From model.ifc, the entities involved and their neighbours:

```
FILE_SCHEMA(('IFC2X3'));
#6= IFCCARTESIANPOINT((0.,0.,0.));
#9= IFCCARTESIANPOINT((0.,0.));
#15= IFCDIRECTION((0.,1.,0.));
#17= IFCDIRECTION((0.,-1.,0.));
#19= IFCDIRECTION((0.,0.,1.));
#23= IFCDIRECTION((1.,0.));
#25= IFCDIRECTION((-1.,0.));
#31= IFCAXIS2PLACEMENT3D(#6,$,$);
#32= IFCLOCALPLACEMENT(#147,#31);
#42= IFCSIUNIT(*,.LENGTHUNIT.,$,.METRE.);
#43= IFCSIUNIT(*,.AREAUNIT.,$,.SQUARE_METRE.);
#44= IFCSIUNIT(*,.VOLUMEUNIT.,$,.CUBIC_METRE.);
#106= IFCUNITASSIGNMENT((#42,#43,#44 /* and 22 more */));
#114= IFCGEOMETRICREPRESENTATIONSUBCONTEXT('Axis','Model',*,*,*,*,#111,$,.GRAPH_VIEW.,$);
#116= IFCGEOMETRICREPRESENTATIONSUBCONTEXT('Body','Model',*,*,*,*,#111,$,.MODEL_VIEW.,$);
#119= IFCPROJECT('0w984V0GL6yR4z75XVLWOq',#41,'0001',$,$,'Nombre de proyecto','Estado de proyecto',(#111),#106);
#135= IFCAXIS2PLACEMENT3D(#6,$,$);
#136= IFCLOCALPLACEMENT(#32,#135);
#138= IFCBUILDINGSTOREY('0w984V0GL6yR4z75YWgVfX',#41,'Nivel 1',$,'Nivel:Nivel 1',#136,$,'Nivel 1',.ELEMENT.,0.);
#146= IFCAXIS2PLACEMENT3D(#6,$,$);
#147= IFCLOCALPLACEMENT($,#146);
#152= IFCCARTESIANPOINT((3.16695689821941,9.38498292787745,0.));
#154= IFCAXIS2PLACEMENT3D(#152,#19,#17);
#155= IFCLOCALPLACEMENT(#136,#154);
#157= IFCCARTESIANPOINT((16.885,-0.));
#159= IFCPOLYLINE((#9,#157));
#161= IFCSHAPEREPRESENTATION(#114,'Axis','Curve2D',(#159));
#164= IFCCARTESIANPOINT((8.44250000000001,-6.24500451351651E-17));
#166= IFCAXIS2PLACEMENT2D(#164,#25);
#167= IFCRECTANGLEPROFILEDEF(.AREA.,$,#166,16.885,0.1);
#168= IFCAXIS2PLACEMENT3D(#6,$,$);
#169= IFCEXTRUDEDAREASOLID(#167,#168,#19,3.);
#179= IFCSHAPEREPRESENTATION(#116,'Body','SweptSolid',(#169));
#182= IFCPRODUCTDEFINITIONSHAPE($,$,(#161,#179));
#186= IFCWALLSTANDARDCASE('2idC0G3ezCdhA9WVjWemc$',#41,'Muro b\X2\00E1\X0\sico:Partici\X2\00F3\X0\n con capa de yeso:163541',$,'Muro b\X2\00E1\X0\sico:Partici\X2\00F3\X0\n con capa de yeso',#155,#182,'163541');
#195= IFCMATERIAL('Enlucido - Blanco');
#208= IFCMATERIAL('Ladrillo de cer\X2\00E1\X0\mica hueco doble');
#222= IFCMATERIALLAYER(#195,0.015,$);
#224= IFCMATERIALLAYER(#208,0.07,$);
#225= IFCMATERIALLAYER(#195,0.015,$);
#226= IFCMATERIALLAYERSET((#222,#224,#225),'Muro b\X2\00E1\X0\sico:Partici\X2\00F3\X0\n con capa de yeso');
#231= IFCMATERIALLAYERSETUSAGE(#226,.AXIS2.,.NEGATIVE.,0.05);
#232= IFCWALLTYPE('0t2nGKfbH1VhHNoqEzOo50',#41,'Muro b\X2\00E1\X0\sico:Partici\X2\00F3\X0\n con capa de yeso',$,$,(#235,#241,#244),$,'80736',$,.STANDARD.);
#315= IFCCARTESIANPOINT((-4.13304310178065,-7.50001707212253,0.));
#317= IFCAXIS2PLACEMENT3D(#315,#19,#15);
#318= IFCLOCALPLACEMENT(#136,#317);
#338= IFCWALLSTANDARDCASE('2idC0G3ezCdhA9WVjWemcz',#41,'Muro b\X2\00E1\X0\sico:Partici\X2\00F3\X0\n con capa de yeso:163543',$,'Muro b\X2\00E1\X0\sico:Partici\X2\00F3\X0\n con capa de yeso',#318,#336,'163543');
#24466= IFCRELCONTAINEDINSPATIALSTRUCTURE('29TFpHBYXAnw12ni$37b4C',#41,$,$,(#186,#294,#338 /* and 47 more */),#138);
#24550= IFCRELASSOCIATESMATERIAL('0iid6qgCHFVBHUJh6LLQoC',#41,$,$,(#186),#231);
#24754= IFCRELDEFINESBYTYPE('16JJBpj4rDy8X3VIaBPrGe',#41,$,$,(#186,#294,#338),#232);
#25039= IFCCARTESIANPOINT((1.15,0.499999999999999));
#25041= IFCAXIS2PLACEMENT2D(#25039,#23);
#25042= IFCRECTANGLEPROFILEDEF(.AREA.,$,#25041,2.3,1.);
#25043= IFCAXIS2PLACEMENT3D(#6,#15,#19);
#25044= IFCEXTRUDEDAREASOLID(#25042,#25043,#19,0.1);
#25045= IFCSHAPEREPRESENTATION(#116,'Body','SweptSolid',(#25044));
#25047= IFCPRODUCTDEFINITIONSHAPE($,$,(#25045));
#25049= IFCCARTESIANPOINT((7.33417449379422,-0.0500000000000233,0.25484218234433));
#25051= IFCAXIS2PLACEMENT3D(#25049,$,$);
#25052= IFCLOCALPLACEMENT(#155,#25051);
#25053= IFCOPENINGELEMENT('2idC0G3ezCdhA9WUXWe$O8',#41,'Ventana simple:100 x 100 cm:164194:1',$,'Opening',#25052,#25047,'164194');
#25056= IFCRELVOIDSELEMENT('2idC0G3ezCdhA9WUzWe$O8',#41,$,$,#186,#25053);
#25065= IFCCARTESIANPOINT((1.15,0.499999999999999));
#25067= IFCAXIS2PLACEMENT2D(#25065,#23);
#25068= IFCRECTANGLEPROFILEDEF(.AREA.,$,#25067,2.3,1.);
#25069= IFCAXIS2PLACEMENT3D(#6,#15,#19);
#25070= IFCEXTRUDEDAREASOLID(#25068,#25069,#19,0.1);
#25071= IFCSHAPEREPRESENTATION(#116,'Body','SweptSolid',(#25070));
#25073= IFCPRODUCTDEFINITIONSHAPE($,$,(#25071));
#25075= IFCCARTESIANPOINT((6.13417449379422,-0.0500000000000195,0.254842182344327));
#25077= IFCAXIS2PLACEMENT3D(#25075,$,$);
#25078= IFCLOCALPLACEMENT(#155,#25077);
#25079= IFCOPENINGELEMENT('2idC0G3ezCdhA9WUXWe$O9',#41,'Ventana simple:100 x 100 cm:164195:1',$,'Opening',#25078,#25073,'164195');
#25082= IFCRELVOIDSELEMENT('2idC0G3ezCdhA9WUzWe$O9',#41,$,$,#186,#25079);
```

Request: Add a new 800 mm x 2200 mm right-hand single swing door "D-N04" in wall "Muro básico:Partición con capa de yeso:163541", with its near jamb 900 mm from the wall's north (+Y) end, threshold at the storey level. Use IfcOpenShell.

```python
import numpy as np
import ifcopenshell
import ifcopenshell.api.feature
import ifcopenshell.api.geometry
import ifcopenshell.api.root
import ifcopenshell.api.spatial
import ifcopenshell.api.type
import ifcopenshell.geom
import ifcopenshell.util.element
import ifcopenshell.util.placement
import ifcopenshell.util.representation
import ifcopenshell.util.shape
import ifcopenshell.util.unit

model = ifcopenshell.open("model.ifc")
unit_scale = ifcopenshell.util.unit.calculate_unit_scale(model)
settings = ifcopenshell.geom.settings()


def volume(element):
    """Net volume in cubic metres, openings subtracted."""
    shape = ifcopenshell.geom.create_shape(settings, element)
    return ifcopenshell.util.shape.get_volume(shape.geometry)


wall = model.by_guid("2idC0G3ezCdhA9WVjWemc$")
storey = ifcopenshell.util.element.get_container(wall, ifc_class="IfcBuildingStorey")
context = ifcopenshell.util.representation.get_context(model, "Model", "Body", "MODEL_VIEW")
before = volume(wall)

width, height, from_end, sill = 0.8, 2.2, 0.9, 0.0  # metres

# The wall runs along its own X axis, and the end named is its -X end.
wall_shape = ifcopenshell.geom.create_shape(settings, wall)
x, y, z = ifcopenshell.util.shape.get_vertices(wall_shape.geometry).T
start = x.min() + from_end
face, thickness = float(y.min()), float(y.max() - y.min())
wall_matrix = ifcopenshell.util.placement.get_local_placement(wall.ObjectPlacement)
level = ifcopenshell.util.placement.get_local_placement(storey.ObjectPlacement)[2, 3]


def in_wall(x, y):
    """Placement at x, y metres in the wall's axes, at sill height."""
    matrix = wall_matrix.copy()
    matrix[:, 3] = wall_matrix @ np.array([x / unit_scale, y / unit_scale, 0.0, 1.0])
    matrix[2, 3] = level + sill / unit_scale
    return matrix


# Opening: a box that overshoots both wall faces by 50 mm.
opening = ifcopenshell.api.root.create_entity(model, ifc_class="IfcOpeningElement")
box = ifcopenshell.api.geometry.add_wall_representation(
    model, context=context, length=width, height=height, thickness=thickness + 0.1
)
ifcopenshell.api.geometry.assign_representation(model, product=opening, representation=box)
ifcopenshell.api.geometry.edit_object_placement(model, product=opening, matrix=in_wall(start, face - 0.05), is_si=False)
ifcopenshell.api.feature.add_feature(model, feature=opening, element=wall)

door = ifcopenshell.api.root.create_entity(model, ifc_class="IfcDoor", name="D-N04")
door.OverallWidth, door.OverallHeight = width / unit_scale, height / unit_scale
body = ifcopenshell.api.geometry.add_door_representation(
    model,
    context=context,
    overall_width=door.OverallWidth,
    overall_height=door.OverallHeight,
    operation_type="SINGLE_SWING_RIGHT",
    lining_properties={"LiningDepth": thickness / unit_scale, "ThresholdDepth": thickness / unit_scale},
)
ifcopenshell.api.geometry.assign_representation(model, product=door, representation=body)
ifcopenshell.api.spatial.assign_container(model, products=[door], relating_structure=storey)
fills = ifcopenshell.api.feature.add_filling(model, opening=opening, element=door)
fills.OwnerHistory = door.OwnerHistory  # required in IFC2X3

# IFC2X3 keeps the operation on the door style.
style = ifcopenshell.api.root.create_entity(model, ifc_class="IfcDoorStyle", name="D-N04")
style.OperationType, style.ConstructionType = "SINGLE_SWING_RIGHT", "NOTDEFINED"
style.ParameterTakesPrecedence = style.Sizeable = False
ifcopenshell.api.type.assign_type(model, related_objects=[door], relating_type=style)

# The lining spans the wall, so the door starts at the wall face.
ifcopenshell.api.geometry.edit_object_placement(model, product=door, matrix=in_wall(start, face), is_si=False)

after = volume(wall)

print(f"wall volume {before:.3f} -> {after:.3f} m3")

model.write("model-out.ifc")
```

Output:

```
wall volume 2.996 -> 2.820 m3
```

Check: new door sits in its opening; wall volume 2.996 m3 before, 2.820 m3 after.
